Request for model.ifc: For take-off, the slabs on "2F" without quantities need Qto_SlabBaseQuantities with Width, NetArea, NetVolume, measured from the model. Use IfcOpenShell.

First a look at what the model holds.

```python
import ifcopenshell
import ifcopenshell.util.element
import ifcopenshell.util.unit

model = ifcopenshell.open("model.ifc")
print(model.schema)
for unit_type in ("LENGTHUNIT", "AREAUNIT", "VOLUMEUNIT"):
    print(unit_type, ifcopenshell.util.unit.calculate_unit_scale(model, unit_type))
storey = next(s for s in model.by_type("IfcBuildingStorey") if s.Name == "2F")
slabs = [e for e in ifcopenshell.util.element.get_decomposition(storey) if e.is_a("IfcSlab")]
for e in sorted(slabs, key=lambda e: e.id()):
    print(e.id(), e.is_a(), e.Name, list(ifcopenshell.util.element.get_psets(e, qtos_only=True)), sep=" | ")
```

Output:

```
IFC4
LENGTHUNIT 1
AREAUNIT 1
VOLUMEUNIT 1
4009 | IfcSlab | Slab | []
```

```python
import ifcopenshell
import ifcopenshell.api.pset
import ifcopenshell.geom
import ifcopenshell.util.element
import ifcopenshell.util.shape
import ifcopenshell.util.unit

model = ifcopenshell.open("model.ifc")
unit_scale = ifcopenshell.util.unit.calculate_unit_scale(model)
area_scale = ifcopenshell.util.unit.calculate_unit_scale(model, "AREAUNIT")
volume_scale = ifcopenshell.util.unit.calculate_unit_scale(model, "VOLUMEUNIT")
settings = ifcopenshell.geom.settings()

storey = next(s for s in model.by_type("IfcBuildingStorey") if s.Name == "2F")
slabs = [e for e in ifcopenshell.util.element.get_decomposition(storey) if e.is_a("IfcSlab")]

for e in sorted(slabs, key=lambda e: e.id()):
    if ifcopenshell.util.element.get_psets(e, qtos_only=True, should_inherit=False):
        continue
    # Geometry comes back in metres, in the element's own axes.
    shape = ifcopenshell.geom.create_shape(settings, e)
    values = {
        "Width": ifcopenshell.util.shape.get_z(shape.geometry) / unit_scale,
        "NetArea": ifcopenshell.util.shape.get_footprint_area(shape.geometry) / area_scale,
        "NetVolume": ifcopenshell.util.shape.get_volume(shape.geometry) / volume_scale,
    }
    qto = ifcopenshell.api.pset.add_qto(model, product=e, name="Qto_SlabBaseQuantities")
    ifcopenshell.api.pset.edit_qto(model, qto=qto, properties=values)
    print(e.id(), {k: round(v, 3) for k, v in values.items()})

model.write("model_edited.ifc")
```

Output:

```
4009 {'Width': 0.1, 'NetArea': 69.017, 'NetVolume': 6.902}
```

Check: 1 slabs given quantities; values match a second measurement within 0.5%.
